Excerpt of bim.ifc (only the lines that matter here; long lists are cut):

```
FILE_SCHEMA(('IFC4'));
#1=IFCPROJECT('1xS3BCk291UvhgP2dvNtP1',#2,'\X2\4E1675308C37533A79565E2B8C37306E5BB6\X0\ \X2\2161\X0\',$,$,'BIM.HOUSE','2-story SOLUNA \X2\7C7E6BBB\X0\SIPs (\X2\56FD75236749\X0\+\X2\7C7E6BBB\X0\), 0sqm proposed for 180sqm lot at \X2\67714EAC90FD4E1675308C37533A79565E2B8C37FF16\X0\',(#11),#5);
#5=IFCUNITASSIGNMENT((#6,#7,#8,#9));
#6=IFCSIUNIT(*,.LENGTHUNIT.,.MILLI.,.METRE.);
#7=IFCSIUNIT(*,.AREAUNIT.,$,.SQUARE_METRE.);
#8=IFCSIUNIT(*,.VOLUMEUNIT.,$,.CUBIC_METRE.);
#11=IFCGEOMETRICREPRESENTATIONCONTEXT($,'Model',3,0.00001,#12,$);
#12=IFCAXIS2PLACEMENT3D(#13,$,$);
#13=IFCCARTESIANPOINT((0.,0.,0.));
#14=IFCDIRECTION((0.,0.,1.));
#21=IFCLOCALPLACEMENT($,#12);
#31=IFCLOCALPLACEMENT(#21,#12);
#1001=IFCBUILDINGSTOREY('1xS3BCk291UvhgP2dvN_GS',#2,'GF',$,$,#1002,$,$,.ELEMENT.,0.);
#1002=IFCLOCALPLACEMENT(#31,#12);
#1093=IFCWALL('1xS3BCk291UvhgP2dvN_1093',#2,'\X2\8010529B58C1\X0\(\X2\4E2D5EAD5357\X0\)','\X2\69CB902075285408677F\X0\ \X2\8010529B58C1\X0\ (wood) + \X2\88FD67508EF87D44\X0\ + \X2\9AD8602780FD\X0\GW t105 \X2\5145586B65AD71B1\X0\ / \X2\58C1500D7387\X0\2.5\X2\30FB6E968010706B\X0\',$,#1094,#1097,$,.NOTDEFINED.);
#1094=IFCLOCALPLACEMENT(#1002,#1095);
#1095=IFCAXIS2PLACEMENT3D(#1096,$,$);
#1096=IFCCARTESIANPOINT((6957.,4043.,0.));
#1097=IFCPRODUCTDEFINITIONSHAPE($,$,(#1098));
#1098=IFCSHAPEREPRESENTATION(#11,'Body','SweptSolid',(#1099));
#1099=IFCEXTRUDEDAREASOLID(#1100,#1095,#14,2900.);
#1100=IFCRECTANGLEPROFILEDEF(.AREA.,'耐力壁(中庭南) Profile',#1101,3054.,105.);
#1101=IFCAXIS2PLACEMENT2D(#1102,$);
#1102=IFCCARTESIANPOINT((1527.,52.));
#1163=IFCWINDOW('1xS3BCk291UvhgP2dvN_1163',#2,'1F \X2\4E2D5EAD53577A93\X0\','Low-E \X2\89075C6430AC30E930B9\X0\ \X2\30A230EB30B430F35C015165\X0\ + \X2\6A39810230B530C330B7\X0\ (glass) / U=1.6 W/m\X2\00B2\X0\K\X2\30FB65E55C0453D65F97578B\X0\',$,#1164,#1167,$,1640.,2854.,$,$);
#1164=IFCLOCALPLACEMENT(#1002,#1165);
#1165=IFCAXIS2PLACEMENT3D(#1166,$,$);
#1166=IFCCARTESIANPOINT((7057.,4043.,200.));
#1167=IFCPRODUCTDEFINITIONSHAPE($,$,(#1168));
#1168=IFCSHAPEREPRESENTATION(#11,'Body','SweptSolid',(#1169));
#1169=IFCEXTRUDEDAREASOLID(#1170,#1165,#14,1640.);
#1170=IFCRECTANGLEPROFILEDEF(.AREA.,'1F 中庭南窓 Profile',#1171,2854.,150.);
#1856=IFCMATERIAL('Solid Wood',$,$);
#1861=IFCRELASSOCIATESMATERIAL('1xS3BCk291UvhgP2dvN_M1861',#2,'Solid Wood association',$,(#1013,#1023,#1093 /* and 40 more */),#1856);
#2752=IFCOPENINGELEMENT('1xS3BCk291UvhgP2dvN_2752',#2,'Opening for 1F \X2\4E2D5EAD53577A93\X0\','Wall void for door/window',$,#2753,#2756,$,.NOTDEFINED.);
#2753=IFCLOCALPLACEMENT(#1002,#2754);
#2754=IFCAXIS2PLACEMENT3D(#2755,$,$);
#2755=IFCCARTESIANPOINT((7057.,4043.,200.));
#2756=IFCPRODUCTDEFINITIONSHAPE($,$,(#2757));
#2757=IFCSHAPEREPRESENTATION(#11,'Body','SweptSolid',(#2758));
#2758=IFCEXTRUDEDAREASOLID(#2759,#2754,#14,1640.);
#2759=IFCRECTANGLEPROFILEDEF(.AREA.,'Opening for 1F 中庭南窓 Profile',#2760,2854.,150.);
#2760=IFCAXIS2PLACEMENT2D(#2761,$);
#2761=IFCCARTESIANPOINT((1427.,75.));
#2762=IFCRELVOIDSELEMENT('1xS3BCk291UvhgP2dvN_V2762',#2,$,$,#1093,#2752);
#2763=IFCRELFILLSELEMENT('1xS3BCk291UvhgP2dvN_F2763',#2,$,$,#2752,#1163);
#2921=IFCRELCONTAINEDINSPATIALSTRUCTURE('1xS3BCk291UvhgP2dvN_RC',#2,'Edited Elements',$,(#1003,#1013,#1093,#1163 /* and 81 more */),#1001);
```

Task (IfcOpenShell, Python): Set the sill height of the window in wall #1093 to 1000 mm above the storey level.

```python
import numpy as np
import ifcopenshell
import ifcopenshell.api.geometry
import ifcopenshell.geom
import ifcopenshell.util.element
import ifcopenshell.util.placement
import ifcopenshell.util.shape
import ifcopenshell.util.unit

model = ifcopenshell.open("bim.ifc")
unit_scale = ifcopenshell.util.unit.calculate_unit_scale(model)

window = model.by_id(1163)
opening = window.FillsVoids[0].RelatingOpeningElement
storey = ifcopenshell.util.element.get_container(window, ifc_class="IfcBuildingStorey")
level = ifcopenshell.util.placement.get_local_placement(storey.ObjectPlacement)[2, 3]

# The opening's origin need not be at the sill, so measure its lowest point.
shape = ifcopenshell.geom.create_shape(ifcopenshell.geom.settings(), opening)
bottom = ifcopenshell.util.shape.get_shape_bottom_elevation(shape, shape.geometry) / unit_scale
dz = level + 1000.0 - bottom

shift = np.array([0.0, 0.0, dz])
# The window is not placed relative to its opening, so move both.
for product in (opening, window):
    matrix = ifcopenshell.util.placement.get_local_placement(product.ObjectPlacement)
    matrix[:3, 3] += shift
    ifcopenshell.api.geometry.edit_object_placement(model, product=product, matrix=matrix, is_si=False)

print(f"moved by {dz * unit_scale:+.3f} m")

model.write("bim_rev.ifc")
```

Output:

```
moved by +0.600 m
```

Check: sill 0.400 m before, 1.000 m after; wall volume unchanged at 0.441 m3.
